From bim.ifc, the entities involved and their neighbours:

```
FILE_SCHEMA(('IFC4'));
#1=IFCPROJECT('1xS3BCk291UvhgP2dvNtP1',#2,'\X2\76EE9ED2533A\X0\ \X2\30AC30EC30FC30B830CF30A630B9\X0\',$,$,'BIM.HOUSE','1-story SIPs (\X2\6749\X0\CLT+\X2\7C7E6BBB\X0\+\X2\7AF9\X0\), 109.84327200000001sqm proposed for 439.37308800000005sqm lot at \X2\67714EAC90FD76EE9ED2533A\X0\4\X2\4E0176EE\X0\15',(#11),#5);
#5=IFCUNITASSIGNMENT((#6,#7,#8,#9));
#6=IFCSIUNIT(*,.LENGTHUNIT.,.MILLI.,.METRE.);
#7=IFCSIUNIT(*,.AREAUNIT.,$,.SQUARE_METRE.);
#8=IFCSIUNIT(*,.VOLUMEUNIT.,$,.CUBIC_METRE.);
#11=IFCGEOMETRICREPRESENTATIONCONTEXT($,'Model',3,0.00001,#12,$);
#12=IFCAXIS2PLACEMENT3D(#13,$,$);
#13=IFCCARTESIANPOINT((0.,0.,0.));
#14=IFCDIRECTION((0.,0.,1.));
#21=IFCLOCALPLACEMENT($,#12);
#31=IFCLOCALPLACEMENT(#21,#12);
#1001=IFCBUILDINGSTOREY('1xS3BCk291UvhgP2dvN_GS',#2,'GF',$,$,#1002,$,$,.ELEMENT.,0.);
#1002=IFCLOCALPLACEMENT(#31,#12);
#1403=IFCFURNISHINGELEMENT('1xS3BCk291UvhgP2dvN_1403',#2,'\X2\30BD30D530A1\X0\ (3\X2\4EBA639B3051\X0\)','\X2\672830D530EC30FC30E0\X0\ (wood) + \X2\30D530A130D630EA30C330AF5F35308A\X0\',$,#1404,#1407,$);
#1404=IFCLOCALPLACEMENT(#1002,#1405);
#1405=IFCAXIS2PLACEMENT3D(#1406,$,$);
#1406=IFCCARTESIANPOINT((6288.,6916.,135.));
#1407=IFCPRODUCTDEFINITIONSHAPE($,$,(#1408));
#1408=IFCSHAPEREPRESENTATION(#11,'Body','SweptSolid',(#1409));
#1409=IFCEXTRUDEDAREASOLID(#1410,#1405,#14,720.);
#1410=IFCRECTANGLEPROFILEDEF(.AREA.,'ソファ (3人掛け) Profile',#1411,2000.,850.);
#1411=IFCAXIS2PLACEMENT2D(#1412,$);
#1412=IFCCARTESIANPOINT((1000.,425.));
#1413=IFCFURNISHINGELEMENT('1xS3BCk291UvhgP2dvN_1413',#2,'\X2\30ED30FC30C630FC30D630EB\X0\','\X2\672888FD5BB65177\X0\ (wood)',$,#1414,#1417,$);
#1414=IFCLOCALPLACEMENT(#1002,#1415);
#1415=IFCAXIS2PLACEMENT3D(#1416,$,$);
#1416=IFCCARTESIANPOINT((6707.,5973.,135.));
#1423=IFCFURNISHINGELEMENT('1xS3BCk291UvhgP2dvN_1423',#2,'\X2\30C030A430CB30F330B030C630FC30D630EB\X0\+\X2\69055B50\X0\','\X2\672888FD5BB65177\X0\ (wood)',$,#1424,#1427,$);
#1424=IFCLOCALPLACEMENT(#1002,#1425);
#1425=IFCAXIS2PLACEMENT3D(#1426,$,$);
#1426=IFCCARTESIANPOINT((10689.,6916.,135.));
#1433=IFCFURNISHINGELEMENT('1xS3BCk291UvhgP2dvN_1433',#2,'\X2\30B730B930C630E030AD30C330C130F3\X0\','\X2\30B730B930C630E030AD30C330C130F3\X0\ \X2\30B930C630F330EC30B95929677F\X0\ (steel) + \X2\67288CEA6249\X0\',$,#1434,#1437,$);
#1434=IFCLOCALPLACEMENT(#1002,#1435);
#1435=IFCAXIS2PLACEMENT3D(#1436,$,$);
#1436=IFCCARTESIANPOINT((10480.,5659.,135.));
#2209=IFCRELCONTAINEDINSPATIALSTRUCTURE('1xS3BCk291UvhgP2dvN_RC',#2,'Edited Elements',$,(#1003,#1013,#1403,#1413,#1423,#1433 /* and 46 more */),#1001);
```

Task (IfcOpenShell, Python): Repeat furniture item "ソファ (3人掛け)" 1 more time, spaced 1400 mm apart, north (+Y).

```python
import numpy as np
import ifcopenshell
import ifcopenshell.api.geometry
import ifcopenshell.api.root
import ifcopenshell.util.element
import ifcopenshell.util.placement

model = ifcopenshell.open("bim.ifc")


def reuse_history(source, copy):
    """copy_class also copies each property set's owner history, people and application; keep the originals."""
    for rel in copy.IsDefinedBy:
        if rel.is_a("IfcRelDefinesByProperties") and (history := rel.RelatingPropertyDefinition.OwnerHistory):
            rel.RelatingPropertyDefinition.OwnerHistory = source.OwnerHistory
            ifcopenshell.util.element.remove_deep2(model, history)


source = model.by_guid("1xS3BCk291UvhgP2dvN_1403")
base = ifcopenshell.util.placement.get_local_placement(source.ObjectPlacement)
step = np.array([0.0, 1.0, 0.0]) * 1400.0

for i in range(1, 2):
    copy = ifcopenshell.api.root.copy_class(model, product=source)
    copy.Representation = ifcopenshell.util.element.copy_deep(
        model, source.Representation, exclude=["IfcGeometricRepresentationContext", "IfcRepresentationMap"]
    )
    reuse_history(source, copy)
    matrix = base.copy()
    matrix[:3, 3] += i * step
    print("added at", matrix[:3, 3].round(3) + 0.0)
    ifcopenshell.api.geometry.edit_object_placement(model, product=copy, matrix=matrix, is_si=False)

model.write("bim_v2.ifc")
```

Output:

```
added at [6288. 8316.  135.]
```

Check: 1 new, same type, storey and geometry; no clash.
